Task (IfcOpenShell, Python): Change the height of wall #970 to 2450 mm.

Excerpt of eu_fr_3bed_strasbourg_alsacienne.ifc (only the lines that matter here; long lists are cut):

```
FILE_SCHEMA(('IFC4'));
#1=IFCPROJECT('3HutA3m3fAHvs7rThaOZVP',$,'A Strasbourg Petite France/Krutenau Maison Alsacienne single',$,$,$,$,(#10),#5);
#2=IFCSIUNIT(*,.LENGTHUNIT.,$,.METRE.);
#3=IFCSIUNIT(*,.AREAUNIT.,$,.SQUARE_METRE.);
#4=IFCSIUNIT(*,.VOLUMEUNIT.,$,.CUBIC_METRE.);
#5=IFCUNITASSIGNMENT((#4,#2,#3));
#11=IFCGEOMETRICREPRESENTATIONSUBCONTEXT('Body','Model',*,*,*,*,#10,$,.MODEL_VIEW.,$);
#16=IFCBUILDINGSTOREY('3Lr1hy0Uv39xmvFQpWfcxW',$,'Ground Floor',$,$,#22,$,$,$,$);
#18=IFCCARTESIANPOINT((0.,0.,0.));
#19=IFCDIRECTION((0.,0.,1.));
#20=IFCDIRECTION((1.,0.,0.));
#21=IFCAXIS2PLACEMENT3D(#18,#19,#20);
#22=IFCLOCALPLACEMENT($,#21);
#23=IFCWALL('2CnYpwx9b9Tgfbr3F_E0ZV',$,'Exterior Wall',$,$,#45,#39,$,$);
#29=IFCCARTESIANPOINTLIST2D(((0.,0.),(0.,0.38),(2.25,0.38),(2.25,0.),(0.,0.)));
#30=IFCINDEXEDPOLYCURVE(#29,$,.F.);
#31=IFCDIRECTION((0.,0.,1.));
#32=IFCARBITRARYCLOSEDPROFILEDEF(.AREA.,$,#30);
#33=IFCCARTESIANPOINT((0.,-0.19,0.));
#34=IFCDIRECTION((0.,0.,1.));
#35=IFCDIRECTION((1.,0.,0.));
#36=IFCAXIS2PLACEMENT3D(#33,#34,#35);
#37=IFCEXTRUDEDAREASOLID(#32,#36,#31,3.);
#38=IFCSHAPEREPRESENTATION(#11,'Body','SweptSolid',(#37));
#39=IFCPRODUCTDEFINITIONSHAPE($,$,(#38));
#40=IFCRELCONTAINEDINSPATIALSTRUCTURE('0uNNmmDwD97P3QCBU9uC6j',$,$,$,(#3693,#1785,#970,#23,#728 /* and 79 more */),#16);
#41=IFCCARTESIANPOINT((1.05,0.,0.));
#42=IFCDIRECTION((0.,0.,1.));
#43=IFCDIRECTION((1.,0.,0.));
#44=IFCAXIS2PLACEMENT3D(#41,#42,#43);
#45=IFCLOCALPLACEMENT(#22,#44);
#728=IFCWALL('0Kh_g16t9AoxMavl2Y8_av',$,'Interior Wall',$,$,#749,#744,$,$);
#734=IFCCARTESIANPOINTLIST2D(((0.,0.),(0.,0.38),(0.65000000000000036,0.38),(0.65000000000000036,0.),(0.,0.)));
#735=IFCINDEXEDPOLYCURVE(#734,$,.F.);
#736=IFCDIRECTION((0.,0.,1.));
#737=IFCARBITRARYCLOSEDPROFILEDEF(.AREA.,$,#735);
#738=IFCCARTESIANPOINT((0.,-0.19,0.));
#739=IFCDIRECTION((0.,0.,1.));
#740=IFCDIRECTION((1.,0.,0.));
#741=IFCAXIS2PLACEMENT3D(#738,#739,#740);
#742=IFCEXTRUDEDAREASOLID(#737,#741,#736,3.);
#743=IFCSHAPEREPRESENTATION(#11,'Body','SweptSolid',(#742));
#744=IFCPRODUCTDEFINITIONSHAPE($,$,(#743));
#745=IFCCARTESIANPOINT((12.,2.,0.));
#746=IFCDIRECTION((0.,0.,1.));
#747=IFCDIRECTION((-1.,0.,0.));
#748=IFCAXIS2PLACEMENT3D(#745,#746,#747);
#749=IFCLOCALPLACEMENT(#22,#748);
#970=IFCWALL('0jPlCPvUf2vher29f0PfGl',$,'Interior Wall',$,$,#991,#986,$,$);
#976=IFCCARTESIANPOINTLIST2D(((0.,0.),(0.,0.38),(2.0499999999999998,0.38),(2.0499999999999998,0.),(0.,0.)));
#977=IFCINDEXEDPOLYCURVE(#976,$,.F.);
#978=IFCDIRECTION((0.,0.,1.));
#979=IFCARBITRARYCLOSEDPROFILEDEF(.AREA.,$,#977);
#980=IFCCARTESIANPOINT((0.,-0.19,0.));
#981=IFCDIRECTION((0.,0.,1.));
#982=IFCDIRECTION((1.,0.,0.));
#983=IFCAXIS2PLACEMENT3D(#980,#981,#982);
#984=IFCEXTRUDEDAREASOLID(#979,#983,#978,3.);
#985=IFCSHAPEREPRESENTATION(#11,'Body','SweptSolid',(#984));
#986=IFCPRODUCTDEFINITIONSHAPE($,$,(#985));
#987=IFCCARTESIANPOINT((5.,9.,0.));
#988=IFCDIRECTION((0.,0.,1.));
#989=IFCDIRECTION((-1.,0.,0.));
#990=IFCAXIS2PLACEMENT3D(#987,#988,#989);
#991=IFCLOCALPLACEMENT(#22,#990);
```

```python
import ifcopenshell
import ifcopenshell.geom
import ifcopenshell.util.representation
import ifcopenshell.util.shape

model = ifcopenshell.open("eu_fr_3bed_strasbourg_alsacienne.ifc")
settings = ifcopenshell.geom.settings()


def volume(element):
    """Net volume in cubic metres, openings subtracted."""
    shape = ifcopenshell.geom.create_shape(settings, element)
    return ifcopenshell.util.shape.get_volume(shape.geometry)


wall = model.by_guid("0jPlCPvUf2vher29f0PfGl")
before = volume(wall)

body = ifcopenshell.util.representation.get_representation(wall, "Model", "Body")
solid = body.Items[0]
old_height = solid.Depth
solid.Depth = 2.45
after = volume(wall)

print(f"height {old_height:g} -> {solid.Depth:g}, volume {before:.3f} -> {after:.3f} m3")

model.write("eu_fr_3bed_strasbourg_alsacienne-out.ifc")
```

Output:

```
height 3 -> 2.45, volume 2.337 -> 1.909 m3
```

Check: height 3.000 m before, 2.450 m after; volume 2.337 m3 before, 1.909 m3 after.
